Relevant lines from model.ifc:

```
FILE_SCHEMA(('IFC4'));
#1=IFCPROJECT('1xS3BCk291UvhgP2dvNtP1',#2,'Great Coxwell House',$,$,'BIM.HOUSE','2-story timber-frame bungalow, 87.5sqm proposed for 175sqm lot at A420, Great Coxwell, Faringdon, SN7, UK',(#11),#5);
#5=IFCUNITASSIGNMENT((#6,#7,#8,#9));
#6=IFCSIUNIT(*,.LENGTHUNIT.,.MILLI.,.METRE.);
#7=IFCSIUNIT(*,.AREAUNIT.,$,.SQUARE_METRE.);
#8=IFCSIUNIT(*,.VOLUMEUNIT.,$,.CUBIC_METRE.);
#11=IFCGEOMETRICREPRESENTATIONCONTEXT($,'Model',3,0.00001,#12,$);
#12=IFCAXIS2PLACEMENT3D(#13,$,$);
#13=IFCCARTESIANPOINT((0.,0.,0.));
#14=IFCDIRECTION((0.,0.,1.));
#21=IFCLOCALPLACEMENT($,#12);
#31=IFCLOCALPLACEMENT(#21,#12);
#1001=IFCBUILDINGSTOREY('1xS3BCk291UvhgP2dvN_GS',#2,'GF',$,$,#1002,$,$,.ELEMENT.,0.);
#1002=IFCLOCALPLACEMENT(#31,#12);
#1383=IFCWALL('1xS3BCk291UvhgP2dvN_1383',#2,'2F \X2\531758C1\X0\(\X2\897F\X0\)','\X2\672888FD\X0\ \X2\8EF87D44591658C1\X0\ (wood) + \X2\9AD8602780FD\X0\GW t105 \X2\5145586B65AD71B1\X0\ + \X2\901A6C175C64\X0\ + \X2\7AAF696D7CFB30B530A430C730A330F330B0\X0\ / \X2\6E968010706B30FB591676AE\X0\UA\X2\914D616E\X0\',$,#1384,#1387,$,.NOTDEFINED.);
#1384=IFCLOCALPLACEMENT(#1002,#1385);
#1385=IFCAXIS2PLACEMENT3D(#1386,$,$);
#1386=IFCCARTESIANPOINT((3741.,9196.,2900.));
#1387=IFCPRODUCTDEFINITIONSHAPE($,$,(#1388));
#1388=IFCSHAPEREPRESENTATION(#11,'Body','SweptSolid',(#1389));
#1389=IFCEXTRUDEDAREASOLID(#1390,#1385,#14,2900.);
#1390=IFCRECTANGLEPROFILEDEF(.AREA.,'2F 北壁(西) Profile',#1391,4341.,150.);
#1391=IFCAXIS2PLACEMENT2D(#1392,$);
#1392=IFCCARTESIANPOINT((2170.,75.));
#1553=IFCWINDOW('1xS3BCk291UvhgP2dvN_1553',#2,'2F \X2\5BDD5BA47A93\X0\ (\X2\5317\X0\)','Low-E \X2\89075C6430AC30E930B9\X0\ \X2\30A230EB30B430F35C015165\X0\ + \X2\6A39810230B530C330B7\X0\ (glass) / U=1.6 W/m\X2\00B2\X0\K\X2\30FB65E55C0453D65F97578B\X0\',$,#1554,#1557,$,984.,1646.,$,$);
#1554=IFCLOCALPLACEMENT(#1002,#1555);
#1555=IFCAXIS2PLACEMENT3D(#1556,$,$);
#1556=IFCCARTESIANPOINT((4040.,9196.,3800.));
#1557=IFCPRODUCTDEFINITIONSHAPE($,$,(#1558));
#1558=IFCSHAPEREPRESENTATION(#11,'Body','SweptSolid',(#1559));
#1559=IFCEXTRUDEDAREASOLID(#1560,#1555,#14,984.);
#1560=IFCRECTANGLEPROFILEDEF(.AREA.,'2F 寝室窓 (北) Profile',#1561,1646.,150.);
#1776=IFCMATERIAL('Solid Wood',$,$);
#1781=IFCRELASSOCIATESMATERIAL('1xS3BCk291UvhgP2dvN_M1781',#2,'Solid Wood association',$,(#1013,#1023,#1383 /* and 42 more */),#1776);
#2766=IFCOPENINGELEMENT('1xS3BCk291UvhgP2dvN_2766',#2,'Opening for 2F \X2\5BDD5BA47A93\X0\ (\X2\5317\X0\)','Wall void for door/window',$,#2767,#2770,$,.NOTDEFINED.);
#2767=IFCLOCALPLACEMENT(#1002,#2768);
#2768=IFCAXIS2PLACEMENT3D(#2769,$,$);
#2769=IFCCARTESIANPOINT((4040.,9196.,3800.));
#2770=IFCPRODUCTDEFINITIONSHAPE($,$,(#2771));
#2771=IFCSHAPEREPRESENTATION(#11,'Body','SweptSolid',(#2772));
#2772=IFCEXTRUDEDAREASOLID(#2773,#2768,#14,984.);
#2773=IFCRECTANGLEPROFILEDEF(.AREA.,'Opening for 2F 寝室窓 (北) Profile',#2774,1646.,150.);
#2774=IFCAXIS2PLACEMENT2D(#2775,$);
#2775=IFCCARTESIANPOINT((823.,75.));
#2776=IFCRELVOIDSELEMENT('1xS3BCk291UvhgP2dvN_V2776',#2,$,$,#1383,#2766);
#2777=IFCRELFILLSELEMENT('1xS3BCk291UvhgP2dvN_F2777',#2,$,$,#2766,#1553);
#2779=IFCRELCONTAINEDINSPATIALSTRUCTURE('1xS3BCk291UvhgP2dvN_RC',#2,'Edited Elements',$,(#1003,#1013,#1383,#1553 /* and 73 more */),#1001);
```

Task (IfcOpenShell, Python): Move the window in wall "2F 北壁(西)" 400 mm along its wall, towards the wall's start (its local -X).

```python
import ifcopenshell
import ifcopenshell.api.geometry
import ifcopenshell.util.placement
import ifcopenshell.util.unit

model = ifcopenshell.open("model.ifc")
unit_scale = ifcopenshell.util.unit.calculate_unit_scale(model)

window = model.by_guid("1xS3BCk291UvhgP2dvN_1553")
opening = window.FillsVoids[0].RelatingOpeningElement
wall = opening.VoidsElements[0].RelatingBuildingElement

wall_matrix = ifcopenshell.util.placement.get_local_placement(wall.ObjectPlacement)
shift = wall_matrix[:3, 0] * -0.4 / unit_scale
before = ifcopenshell.util.placement.get_local_placement(window.ObjectPlacement)[:3, 3].copy()

# The window is not placed relative to its opening, so move both.
for product in (opening, window):
    matrix = ifcopenshell.util.placement.get_local_placement(product.ObjectPlacement)
    matrix[:3, 3] += shift
    ifcopenshell.api.geometry.edit_object_placement(model, product=product, matrix=matrix, is_si=False)

after = ifcopenshell.util.placement.get_local_placement(window.ObjectPlacement)[:3, 3]
print("window moved by", (after - before).round(3) + 0.0)

model.write("model_updated.ifc")
```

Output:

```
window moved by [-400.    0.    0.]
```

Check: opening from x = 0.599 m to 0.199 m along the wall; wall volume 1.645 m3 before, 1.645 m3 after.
